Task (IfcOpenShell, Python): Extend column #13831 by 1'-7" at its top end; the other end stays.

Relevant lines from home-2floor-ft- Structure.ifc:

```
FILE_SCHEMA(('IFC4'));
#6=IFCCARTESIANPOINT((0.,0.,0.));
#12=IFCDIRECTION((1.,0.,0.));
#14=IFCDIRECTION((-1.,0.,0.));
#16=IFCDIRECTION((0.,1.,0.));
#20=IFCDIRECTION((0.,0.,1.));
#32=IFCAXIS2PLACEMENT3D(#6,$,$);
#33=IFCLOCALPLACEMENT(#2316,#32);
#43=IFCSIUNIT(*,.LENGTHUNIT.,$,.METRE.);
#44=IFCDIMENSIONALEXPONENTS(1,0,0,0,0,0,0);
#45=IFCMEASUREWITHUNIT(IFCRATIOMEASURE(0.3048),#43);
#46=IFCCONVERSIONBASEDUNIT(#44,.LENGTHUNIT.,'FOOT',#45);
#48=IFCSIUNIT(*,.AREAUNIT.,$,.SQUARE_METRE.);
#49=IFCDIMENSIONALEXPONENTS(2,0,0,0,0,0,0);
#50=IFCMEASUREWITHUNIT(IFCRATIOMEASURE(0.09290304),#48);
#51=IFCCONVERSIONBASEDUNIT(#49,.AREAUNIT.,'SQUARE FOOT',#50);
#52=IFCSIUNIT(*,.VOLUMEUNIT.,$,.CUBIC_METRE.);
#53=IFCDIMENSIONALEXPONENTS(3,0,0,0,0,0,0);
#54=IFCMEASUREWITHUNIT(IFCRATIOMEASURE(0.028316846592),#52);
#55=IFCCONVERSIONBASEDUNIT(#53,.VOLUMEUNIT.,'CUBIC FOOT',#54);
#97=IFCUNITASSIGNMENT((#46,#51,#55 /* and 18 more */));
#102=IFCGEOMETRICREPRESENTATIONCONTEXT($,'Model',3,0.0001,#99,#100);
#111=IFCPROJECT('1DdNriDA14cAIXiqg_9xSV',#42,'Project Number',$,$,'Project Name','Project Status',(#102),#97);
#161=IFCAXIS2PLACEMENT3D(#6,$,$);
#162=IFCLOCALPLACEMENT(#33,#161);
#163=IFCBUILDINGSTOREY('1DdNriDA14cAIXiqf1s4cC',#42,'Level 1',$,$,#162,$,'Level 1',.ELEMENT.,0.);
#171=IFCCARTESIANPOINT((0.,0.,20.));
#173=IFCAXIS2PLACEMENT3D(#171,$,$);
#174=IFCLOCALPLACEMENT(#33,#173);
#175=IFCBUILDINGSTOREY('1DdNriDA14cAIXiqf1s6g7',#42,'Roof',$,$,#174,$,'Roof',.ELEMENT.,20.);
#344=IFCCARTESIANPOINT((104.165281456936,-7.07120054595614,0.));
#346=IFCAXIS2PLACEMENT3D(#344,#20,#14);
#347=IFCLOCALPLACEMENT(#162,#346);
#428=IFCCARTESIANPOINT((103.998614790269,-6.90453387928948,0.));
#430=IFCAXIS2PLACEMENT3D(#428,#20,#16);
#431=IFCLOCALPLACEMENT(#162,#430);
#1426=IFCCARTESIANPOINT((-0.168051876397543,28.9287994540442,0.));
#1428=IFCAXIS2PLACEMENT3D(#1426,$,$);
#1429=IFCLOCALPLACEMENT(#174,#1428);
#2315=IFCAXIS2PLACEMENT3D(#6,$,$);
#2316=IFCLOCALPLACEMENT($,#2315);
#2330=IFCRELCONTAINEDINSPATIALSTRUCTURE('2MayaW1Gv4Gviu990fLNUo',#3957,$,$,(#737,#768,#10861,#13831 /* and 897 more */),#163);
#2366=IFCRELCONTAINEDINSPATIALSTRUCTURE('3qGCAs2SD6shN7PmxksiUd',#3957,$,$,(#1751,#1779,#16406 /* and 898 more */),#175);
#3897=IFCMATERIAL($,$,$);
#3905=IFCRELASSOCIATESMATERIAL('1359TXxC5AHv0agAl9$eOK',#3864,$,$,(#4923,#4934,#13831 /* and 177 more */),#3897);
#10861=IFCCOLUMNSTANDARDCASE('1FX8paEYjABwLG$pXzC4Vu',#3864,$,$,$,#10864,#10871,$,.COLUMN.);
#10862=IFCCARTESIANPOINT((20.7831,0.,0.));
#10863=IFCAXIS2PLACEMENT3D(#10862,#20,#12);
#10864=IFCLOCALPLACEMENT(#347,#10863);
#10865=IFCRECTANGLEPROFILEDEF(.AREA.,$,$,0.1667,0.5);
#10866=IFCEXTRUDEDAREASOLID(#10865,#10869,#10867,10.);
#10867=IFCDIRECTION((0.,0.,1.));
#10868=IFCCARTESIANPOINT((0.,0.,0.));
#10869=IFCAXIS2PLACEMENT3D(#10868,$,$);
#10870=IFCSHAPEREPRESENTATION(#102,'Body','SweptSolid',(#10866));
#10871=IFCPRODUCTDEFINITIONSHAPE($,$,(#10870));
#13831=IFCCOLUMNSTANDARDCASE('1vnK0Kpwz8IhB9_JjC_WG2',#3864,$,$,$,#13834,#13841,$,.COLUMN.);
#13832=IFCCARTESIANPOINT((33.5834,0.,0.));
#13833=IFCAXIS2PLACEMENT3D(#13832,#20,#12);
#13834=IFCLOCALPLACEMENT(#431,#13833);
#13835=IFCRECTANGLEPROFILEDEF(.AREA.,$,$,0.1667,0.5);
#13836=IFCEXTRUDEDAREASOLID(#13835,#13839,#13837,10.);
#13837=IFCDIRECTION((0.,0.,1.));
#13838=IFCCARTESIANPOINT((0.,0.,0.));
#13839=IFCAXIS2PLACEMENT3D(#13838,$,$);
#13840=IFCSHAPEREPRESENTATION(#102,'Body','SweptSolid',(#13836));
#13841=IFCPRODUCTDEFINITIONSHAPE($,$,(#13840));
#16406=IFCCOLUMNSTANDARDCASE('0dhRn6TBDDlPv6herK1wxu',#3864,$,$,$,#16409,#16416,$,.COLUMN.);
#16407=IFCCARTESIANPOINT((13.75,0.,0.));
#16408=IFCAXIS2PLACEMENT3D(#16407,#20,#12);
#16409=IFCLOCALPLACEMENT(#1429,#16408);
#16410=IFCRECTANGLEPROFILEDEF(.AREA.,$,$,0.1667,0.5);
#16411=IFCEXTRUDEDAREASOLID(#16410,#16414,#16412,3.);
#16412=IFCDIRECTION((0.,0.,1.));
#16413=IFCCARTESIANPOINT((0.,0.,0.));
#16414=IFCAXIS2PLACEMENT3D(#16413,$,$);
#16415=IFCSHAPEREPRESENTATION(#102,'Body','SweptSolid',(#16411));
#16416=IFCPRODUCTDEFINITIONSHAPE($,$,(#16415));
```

```python
import ifcopenshell
import ifcopenshell.util.unit

model = ifcopenshell.open("home-2floor-ft- Structure.ifc")
unit_scale = ifcopenshell.util.unit.calculate_unit_scale(model)

member = model.by_guid("1vnK0Kpwz8IhB9_JjC_WG2")
change = 19 * 0.0254 / unit_scale

# The extrusion runs towards the end named, so only its depth changes.
body = next(r for r in member.Representation.Representations if r.RepresentationIdentifier == "Body")
solid = body.Items[0]
old_length = solid.Depth
solid.Depth += change

print(f"length {old_length:g} -> {solid.Depth:g}")

model.write("home-2floor-ft- Structure_updated.ifc")
```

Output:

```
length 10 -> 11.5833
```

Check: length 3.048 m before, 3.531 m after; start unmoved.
